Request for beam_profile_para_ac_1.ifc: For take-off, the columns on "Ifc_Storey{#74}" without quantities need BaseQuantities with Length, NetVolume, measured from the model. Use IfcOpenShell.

First a look at what the model holds.

```python
import ifcopenshell
import ifcopenshell.util.element
import ifcopenshell.util.unit

model = ifcopenshell.open("beam_profile_para_ac_1.ifc")
print(model.schema)
for unit_type in ("LENGTHUNIT", "AREAUNIT", "VOLUMEUNIT"):
    print(unit_type, ifcopenshell.util.unit.calculate_unit_scale(model, unit_type))
storey = next(s for s in model.by_type("IfcBuildingStorey") if s.Name == "Ifc_Storey{#74}")
columns = [e for e in ifcopenshell.util.element.get_decomposition(storey) if e.is_a("IfcColumn")]
for e in sorted(columns, key=lambda e: e.id()):
    print(e.id(), e.is_a(), e.Name, list(ifcopenshell.util.element.get_psets(e, qtos_only=True)), sep=" | ")
```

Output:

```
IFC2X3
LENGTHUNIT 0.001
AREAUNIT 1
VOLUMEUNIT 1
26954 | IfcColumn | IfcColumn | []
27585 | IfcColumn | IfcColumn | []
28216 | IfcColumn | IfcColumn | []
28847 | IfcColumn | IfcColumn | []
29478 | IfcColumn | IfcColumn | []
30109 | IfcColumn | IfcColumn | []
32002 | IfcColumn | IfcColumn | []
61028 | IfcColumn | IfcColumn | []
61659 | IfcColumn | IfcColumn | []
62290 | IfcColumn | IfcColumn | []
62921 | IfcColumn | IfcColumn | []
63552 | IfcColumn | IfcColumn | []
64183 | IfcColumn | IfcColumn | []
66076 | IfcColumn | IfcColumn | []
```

```python
import ifcopenshell
import ifcopenshell.api.pset
import ifcopenshell.geom
import ifcopenshell.util.element
import ifcopenshell.util.shape
import ifcopenshell.util.unit

model = ifcopenshell.open("beam_profile_para_ac_1.ifc")
unit_scale = ifcopenshell.util.unit.calculate_unit_scale(model)
volume_scale = ifcopenshell.util.unit.calculate_unit_scale(model, "VOLUMEUNIT")
settings = ifcopenshell.geom.settings()

storey = next(s for s in model.by_type("IfcBuildingStorey") if s.Name == "Ifc_Storey{#74}")
columns = [e for e in ifcopenshell.util.element.get_decomposition(storey) if e.is_a("IfcColumn")]

for e in sorted(columns, key=lambda e: e.id()):
    if ifcopenshell.util.element.get_psets(e, qtos_only=True, should_inherit=False):
        continue
    # Geometry comes back in metres, in the element's own axes.
    shape = ifcopenshell.geom.create_shape(settings, e)
    values = {
        "Length": ifcopenshell.util.shape.get_z(shape.geometry) / unit_scale,
        "NetVolume": ifcopenshell.util.shape.get_volume(shape.geometry) / volume_scale,
    }
    qto = ifcopenshell.api.pset.add_qto(model, product=e, name="BaseQuantities")
    ifcopenshell.api.pset.edit_qto(model, qto=qto, properties=values)
    print(e.id(), {k: round(v, 3) for k, v in values.items()})

model.write("beam_profile_para_ac_1_edited.ifc")
```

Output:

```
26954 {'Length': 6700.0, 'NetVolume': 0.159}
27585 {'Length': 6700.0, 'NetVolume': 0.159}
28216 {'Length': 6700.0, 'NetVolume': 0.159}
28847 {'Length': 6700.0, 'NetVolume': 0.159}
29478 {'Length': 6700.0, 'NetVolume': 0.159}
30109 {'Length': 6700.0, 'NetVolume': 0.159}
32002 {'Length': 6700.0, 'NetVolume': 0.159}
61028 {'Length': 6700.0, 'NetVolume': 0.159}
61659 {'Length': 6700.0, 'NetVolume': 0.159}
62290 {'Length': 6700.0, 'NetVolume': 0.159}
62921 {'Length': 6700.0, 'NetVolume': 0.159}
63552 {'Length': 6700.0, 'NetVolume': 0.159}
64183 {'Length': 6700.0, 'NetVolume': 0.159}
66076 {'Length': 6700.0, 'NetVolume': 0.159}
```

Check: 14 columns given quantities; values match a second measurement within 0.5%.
